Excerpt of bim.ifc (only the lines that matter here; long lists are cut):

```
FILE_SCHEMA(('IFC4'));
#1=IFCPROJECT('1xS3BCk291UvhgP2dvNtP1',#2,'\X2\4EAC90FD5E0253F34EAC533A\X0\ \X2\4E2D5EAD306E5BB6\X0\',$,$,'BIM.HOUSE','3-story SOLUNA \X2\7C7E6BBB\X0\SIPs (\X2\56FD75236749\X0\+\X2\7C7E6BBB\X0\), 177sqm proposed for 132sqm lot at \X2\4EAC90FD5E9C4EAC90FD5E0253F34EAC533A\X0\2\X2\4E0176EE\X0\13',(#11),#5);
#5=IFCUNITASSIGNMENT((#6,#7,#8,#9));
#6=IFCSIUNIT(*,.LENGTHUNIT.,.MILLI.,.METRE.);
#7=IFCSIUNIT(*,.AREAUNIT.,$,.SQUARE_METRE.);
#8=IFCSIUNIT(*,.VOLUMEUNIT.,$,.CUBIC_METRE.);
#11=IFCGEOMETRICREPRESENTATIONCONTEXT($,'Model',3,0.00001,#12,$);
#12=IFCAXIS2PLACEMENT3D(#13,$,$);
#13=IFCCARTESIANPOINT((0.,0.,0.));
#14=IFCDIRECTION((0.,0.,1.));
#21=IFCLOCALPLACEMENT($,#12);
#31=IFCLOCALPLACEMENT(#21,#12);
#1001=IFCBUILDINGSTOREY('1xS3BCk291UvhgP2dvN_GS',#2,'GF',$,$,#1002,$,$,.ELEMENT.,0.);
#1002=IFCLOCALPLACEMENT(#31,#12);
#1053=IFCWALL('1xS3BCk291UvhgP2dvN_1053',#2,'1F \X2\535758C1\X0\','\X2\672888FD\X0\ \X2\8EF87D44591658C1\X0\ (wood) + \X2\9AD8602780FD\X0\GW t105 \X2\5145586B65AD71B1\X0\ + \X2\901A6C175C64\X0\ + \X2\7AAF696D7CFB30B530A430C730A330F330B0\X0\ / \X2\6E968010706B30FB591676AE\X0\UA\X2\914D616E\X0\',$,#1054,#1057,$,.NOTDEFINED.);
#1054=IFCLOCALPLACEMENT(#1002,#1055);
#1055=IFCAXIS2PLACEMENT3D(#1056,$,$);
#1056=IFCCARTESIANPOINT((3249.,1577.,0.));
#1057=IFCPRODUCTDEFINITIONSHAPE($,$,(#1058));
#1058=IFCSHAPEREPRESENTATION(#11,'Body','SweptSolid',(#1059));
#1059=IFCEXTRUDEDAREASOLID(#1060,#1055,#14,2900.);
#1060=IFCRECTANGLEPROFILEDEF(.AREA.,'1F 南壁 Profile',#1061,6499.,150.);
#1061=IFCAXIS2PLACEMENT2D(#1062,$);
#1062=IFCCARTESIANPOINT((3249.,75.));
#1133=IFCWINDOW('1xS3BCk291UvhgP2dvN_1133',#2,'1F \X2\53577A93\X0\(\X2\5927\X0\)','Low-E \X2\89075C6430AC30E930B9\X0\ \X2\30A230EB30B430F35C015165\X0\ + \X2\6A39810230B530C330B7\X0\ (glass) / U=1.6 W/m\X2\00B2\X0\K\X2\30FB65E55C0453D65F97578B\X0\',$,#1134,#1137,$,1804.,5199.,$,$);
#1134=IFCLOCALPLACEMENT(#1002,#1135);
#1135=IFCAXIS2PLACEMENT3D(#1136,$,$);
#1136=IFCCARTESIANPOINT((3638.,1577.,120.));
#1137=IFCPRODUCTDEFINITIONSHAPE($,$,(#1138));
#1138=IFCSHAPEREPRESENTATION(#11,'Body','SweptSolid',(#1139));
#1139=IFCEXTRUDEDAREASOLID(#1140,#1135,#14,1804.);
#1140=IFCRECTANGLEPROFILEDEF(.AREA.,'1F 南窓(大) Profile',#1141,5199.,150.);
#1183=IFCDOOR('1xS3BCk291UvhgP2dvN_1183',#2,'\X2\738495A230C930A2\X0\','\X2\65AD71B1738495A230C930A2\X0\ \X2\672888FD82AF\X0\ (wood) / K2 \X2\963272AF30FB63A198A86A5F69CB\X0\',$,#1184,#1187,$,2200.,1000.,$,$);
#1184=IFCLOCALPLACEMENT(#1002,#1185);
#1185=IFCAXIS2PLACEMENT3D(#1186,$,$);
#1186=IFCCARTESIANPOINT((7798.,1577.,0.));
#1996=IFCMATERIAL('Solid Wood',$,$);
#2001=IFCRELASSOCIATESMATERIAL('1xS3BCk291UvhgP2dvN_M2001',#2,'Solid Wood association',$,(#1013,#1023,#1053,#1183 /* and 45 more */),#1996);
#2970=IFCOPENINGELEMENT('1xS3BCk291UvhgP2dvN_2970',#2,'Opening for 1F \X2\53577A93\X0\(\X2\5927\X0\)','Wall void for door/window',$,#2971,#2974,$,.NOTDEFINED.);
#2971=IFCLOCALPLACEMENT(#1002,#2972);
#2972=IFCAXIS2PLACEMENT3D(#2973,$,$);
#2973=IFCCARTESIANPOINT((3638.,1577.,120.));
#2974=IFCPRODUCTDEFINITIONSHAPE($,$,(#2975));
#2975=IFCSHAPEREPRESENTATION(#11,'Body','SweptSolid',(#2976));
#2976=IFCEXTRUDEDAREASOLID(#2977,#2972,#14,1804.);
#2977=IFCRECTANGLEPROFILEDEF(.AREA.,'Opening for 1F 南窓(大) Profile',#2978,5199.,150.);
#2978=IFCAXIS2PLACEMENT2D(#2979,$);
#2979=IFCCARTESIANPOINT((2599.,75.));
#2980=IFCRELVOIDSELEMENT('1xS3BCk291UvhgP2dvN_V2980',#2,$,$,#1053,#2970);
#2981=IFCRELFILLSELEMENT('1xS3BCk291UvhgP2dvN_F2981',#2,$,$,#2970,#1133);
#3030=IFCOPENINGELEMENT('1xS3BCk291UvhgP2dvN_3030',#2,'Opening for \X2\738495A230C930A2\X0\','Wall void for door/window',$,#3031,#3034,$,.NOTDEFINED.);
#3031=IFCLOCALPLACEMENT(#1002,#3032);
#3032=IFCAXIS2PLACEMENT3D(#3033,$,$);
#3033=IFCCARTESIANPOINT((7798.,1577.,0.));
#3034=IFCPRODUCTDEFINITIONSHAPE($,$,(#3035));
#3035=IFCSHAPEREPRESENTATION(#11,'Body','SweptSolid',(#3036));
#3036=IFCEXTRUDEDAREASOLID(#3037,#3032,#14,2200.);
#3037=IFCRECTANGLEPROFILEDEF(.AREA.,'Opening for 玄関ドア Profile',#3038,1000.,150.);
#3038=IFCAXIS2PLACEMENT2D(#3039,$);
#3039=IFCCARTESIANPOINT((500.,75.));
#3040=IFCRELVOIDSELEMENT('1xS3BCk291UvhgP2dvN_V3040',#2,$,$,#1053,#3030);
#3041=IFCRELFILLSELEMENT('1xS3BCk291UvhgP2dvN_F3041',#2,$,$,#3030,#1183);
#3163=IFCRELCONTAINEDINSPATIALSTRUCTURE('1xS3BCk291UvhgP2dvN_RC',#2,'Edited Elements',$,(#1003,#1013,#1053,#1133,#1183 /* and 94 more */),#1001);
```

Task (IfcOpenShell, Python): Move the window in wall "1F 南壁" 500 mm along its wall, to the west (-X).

```python
import ifcopenshell
import ifcopenshell.api.geometry
import ifcopenshell.util.placement
import ifcopenshell.util.unit

model = ifcopenshell.open("bim.ifc")
unit_scale = ifcopenshell.util.unit.calculate_unit_scale(model)

window = model.by_guid("1xS3BCk291UvhgP2dvN_1133")
opening = window.FillsVoids[0].RelatingOpeningElement
wall = opening.VoidsElements[0].RelatingBuildingElement

wall_matrix = ifcopenshell.util.placement.get_local_placement(wall.ObjectPlacement)
shift = wall_matrix[:3, 0] * -0.5 / unit_scale
before = ifcopenshell.util.placement.get_local_placement(window.ObjectPlacement)[:3, 3].copy()

# The window is not placed relative to its opening, so move both.
for product in (opening, window):
    matrix = ifcopenshell.util.placement.get_local_placement(product.ObjectPlacement)
    matrix[:3, 3] += shift
    ifcopenshell.api.geometry.edit_object_placement(model, product=product, matrix=matrix, is_si=False)

after = ifcopenshell.util.placement.get_local_placement(window.ObjectPlacement)[:3, 3]
print("window moved by", (after - before).round(3) + 0.0)

model.write("bim_updated.ifc")
```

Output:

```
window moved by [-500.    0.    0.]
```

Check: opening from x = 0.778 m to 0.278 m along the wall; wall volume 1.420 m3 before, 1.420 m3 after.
